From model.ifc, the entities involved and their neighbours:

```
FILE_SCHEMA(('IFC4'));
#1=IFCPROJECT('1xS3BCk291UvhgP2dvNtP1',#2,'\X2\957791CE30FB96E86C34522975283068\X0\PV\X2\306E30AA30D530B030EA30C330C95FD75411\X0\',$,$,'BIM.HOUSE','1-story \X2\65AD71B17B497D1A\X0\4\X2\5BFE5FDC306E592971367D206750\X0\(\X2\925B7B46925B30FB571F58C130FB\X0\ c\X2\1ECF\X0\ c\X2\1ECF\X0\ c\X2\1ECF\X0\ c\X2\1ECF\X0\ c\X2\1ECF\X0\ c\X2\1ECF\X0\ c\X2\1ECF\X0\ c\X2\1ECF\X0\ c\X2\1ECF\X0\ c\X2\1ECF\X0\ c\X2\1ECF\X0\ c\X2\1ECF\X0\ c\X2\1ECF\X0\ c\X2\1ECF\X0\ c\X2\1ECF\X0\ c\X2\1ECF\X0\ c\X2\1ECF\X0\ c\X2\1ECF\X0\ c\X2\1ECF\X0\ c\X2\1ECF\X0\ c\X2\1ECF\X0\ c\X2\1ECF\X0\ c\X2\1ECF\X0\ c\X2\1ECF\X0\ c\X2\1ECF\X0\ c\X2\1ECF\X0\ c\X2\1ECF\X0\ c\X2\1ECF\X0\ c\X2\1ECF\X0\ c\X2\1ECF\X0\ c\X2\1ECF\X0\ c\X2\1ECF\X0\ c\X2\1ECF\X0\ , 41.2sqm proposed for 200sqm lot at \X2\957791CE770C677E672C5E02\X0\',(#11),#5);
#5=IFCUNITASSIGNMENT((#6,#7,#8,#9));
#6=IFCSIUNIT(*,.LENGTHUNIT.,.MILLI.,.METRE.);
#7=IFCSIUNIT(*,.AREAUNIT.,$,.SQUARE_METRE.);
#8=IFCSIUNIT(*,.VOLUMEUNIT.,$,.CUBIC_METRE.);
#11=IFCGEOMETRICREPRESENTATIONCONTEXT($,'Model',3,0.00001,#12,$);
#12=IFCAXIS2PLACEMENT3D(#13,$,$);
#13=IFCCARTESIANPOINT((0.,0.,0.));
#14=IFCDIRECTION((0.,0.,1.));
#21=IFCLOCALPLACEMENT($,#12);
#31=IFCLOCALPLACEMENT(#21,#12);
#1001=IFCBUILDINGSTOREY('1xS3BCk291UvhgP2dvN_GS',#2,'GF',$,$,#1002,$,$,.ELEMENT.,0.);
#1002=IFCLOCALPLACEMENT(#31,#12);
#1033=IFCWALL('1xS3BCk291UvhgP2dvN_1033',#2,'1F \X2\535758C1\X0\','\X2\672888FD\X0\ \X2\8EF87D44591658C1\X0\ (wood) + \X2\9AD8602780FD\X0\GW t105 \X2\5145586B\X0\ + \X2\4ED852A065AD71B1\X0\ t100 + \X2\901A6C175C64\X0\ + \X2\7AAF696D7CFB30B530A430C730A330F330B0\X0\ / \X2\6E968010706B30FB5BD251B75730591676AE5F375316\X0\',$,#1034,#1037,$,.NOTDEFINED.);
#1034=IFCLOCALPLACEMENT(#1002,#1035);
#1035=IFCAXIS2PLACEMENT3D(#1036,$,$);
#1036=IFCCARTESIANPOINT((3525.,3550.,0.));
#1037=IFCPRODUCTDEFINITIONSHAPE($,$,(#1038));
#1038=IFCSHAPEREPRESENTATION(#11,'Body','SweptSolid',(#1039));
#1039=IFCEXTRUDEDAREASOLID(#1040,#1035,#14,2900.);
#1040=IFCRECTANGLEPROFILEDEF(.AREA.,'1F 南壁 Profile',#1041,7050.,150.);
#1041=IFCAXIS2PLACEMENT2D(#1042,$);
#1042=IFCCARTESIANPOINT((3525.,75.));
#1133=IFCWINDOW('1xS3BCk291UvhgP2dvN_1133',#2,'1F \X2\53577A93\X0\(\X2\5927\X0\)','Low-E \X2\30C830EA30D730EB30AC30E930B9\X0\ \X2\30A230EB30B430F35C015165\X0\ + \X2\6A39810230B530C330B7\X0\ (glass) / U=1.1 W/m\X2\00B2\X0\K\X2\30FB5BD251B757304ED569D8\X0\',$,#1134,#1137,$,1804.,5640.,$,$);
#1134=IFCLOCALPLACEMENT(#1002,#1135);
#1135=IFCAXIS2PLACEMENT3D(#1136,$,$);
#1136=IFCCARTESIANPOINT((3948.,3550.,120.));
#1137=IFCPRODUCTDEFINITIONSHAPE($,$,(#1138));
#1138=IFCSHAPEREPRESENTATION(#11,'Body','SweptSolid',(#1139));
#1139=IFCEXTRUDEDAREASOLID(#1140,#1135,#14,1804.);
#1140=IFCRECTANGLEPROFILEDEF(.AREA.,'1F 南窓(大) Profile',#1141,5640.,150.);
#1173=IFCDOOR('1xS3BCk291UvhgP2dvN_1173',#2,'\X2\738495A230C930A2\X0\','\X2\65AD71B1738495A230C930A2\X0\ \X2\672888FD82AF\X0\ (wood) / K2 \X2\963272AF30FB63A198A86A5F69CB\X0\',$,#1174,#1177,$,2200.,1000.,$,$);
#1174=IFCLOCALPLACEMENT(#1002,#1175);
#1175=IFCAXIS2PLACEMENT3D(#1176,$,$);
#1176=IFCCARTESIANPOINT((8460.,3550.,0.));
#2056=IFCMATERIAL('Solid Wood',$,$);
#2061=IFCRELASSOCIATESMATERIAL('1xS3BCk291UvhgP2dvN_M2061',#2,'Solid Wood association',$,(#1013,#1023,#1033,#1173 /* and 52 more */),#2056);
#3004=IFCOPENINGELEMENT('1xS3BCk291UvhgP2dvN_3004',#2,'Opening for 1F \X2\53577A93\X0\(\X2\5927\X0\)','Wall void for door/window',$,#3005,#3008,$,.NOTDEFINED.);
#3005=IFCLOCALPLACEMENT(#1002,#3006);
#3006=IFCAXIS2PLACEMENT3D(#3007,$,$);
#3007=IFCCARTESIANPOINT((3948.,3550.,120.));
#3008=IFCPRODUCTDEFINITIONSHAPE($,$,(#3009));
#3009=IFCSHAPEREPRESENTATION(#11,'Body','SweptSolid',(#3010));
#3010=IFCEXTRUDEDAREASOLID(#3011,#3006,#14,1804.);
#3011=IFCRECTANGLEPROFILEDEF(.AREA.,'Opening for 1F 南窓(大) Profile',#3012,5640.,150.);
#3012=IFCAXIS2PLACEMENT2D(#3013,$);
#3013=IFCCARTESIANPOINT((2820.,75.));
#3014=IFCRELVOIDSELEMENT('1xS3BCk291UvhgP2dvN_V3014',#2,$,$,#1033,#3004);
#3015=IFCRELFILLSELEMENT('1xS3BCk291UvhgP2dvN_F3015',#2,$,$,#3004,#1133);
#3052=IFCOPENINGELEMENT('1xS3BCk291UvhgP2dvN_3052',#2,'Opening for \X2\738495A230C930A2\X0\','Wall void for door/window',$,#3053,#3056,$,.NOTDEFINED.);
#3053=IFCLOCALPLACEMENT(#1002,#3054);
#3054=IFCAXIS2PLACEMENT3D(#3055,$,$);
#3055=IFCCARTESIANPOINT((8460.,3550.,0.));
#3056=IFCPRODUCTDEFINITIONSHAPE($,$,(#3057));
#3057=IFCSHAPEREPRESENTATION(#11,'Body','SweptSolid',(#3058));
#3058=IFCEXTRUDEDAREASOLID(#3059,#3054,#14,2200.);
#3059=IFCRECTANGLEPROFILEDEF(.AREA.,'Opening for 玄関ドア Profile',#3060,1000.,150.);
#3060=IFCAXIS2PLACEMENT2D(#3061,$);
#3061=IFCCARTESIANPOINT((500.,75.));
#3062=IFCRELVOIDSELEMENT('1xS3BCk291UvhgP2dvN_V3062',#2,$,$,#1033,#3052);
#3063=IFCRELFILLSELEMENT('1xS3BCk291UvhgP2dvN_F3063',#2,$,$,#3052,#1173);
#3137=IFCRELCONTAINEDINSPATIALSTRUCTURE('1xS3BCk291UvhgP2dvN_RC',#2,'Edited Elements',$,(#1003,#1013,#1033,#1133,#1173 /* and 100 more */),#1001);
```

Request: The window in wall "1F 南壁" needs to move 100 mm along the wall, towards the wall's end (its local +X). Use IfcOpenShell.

```python
import ifcopenshell
import ifcopenshell.api.geometry
import ifcopenshell.util.placement
import ifcopenshell.util.unit

model = ifcopenshell.open("model.ifc")
unit_scale = ifcopenshell.util.unit.calculate_unit_scale(model)

window = model.by_guid("1xS3BCk291UvhgP2dvN_1133")
opening = window.FillsVoids[0].RelatingOpeningElement
wall = opening.VoidsElements[0].RelatingBuildingElement

wall_matrix = ifcopenshell.util.placement.get_local_placement(wall.ObjectPlacement)
shift = wall_matrix[:3, 0] * 0.1 / unit_scale
before = ifcopenshell.util.placement.get_local_placement(window.ObjectPlacement)[:3, 3].copy()

# The window is not placed relative to its opening, so move both.
for product in (opening, window):
    matrix = ifcopenshell.util.placement.get_local_placement(product.ObjectPlacement)
    matrix[:3, 3] += shift
    ifcopenshell.api.geometry.edit_object_placement(model, product=product, matrix=matrix, is_si=False)

after = ifcopenshell.util.placement.get_local_placement(window.ObjectPlacement)[:3, 3]
print("window moved by", (after - before).round(3) + 0.0)

model.write("model_v2.ifc")
```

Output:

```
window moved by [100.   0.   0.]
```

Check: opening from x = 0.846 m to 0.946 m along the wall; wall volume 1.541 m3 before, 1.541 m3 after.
